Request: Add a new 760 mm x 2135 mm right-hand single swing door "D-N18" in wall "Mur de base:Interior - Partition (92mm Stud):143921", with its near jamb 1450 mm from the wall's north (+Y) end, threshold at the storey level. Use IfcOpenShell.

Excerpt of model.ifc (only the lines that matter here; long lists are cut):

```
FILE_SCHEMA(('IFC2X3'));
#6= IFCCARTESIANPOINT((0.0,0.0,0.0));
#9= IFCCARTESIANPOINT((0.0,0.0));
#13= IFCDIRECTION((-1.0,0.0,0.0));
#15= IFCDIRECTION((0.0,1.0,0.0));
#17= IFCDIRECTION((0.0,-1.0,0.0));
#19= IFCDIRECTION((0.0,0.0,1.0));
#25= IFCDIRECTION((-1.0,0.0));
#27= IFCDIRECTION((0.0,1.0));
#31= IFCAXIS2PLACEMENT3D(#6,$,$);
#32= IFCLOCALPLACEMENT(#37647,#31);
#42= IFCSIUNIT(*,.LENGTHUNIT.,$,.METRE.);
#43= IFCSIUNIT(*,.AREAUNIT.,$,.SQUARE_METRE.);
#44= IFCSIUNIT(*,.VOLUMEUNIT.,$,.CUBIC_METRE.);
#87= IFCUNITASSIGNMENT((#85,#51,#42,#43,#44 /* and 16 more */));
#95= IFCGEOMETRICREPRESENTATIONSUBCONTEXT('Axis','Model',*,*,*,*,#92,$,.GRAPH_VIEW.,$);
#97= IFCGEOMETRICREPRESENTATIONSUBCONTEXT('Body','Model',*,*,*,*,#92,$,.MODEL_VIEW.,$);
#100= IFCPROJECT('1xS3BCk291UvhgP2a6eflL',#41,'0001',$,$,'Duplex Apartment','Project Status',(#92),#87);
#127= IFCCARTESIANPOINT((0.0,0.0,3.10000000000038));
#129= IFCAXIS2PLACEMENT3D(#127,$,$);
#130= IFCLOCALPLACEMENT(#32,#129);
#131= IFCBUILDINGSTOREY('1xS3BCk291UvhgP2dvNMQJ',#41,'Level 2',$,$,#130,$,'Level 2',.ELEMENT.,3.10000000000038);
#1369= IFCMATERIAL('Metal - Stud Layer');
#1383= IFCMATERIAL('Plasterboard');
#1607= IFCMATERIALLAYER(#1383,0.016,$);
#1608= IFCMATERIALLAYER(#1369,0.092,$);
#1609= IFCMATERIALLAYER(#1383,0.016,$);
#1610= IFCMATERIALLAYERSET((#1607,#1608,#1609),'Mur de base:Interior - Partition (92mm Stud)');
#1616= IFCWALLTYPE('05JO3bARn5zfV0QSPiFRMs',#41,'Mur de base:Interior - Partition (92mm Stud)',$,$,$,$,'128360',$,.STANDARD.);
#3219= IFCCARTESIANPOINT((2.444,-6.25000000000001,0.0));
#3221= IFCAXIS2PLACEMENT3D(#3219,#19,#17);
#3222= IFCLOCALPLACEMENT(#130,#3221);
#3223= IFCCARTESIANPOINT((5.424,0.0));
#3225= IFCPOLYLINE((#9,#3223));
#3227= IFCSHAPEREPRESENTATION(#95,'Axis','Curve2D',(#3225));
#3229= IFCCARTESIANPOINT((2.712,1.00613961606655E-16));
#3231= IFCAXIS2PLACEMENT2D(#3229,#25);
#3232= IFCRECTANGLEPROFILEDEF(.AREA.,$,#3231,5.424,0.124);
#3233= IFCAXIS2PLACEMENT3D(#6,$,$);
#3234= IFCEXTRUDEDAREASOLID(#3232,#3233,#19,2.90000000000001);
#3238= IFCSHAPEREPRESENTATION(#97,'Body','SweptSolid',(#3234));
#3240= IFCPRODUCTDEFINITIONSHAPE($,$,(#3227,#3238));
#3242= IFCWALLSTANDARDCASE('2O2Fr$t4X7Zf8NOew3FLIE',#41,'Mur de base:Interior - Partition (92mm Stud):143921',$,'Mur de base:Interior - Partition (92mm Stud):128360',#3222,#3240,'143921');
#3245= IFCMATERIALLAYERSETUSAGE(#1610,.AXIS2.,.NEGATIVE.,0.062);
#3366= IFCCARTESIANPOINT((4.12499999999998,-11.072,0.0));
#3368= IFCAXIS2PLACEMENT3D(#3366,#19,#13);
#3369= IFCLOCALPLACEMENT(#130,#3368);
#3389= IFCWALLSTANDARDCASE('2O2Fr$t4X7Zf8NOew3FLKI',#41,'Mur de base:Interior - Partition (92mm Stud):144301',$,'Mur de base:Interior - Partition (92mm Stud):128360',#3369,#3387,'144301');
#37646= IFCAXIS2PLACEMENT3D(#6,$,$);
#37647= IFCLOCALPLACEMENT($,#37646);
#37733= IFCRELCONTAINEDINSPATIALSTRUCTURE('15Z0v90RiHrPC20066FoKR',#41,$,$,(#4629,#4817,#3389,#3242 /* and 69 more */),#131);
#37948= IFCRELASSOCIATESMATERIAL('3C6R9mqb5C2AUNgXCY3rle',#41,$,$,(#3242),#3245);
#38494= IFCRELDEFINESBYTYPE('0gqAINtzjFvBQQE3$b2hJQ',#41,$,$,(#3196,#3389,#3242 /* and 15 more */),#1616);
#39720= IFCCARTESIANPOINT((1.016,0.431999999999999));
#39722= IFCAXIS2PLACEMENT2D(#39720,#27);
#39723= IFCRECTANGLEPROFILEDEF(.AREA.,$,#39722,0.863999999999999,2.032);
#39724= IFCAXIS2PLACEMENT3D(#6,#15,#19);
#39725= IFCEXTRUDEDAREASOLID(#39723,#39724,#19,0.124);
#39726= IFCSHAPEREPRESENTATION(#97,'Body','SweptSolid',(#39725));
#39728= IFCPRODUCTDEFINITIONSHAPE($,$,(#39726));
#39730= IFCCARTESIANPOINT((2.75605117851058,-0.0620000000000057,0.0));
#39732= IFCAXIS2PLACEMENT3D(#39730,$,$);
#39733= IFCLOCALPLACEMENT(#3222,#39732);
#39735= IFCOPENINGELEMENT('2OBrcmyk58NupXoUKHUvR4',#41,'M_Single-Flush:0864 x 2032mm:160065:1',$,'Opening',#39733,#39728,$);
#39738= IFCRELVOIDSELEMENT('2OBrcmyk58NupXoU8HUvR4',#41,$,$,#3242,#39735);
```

```python
import numpy as np
import ifcopenshell
import ifcopenshell.api.feature
import ifcopenshell.api.geometry
import ifcopenshell.api.root
import ifcopenshell.api.spatial
import ifcopenshell.api.type
import ifcopenshell.geom
import ifcopenshell.util.element
import ifcopenshell.util.placement
import ifcopenshell.util.representation
import ifcopenshell.util.shape
import ifcopenshell.util.unit

model = ifcopenshell.open("model.ifc")
unit_scale = ifcopenshell.util.unit.calculate_unit_scale(model)
settings = ifcopenshell.geom.settings()


def volume(element):
    """Net volume in cubic metres, openings subtracted."""
    shape = ifcopenshell.geom.create_shape(settings, element)
    return ifcopenshell.util.shape.get_volume(shape.geometry)


wall = model.by_id(3242)
storey = ifcopenshell.util.element.get_container(wall, ifc_class="IfcBuildingStorey")
context = ifcopenshell.util.representation.get_context(model, "Model", "Body", "MODEL_VIEW")
before = volume(wall)

width, height, from_end, sill = 0.76, 2.135, 1.45, 0.0  # metres

# The wall runs along its own X axis, and the end named is its -X end.
wall_shape = ifcopenshell.geom.create_shape(settings, wall)
x, y, z = ifcopenshell.util.shape.get_vertices(wall_shape.geometry).T
start = x.min() + from_end
face, thickness = float(y.min()), float(y.max() - y.min())
wall_matrix = ifcopenshell.util.placement.get_local_placement(wall.ObjectPlacement)
level = ifcopenshell.util.placement.get_local_placement(storey.ObjectPlacement)[2, 3]


def in_wall(x, y):
    """Placement at x, y metres in the wall's axes, at sill height."""
    matrix = wall_matrix.copy()
    matrix[:, 3] = wall_matrix @ np.array([x / unit_scale, y / unit_scale, 0.0, 1.0])
    matrix[2, 3] = level + sill / unit_scale
    return matrix


# Opening: a box that overshoots both wall faces by 50 mm.
opening = ifcopenshell.api.root.create_entity(model, ifc_class="IfcOpeningElement")
box = ifcopenshell.api.geometry.add_wall_representation(
    model, context=context, length=width, height=height, thickness=thickness + 0.1
)
ifcopenshell.api.geometry.assign_representation(model, product=opening, representation=box)
ifcopenshell.api.geometry.edit_object_placement(model, product=opening, matrix=in_wall(start, face - 0.05), is_si=False)
ifcopenshell.api.feature.add_feature(model, feature=opening, element=wall)

door = ifcopenshell.api.root.create_entity(model, ifc_class="IfcDoor", name="D-N18")
door.OverallWidth, door.OverallHeight = width / unit_scale, height / unit_scale
body = ifcopenshell.api.geometry.add_door_representation(
    model,
    context=context,
    overall_width=door.OverallWidth,
    overall_height=door.OverallHeight,
    operation_type="SINGLE_SWING_RIGHT",
    lining_properties={"LiningDepth": thickness / unit_scale, "ThresholdDepth": thickness / unit_scale},
)
ifcopenshell.api.geometry.assign_representation(model, product=door, representation=body)
ifcopenshell.api.spatial.assign_container(model, products=[door], relating_structure=storey)
fills = ifcopenshell.api.feature.add_filling(model, opening=opening, element=door)
fills.OwnerHistory = door.OwnerHistory  # required in IFC2X3

# IFC2X3 keeps the operation on the door style.
style = ifcopenshell.api.root.create_entity(model, ifc_class="IfcDoorStyle", name="D-N18")
style.OperationType, style.ConstructionType = "SINGLE_SWING_RIGHT", "NOTDEFINED"
style.ParameterTakesPrecedence = style.Sizeable = False
ifcopenshell.api.type.assign_type(model, related_objects=[door], relating_type=style)

# The lining spans the wall, so the door starts at the wall face.
ifcopenshell.api.geometry.edit_object_placement(model, product=door, matrix=in_wall(start, face), is_si=False)

after = volume(wall)

print(f"wall volume {before:.3f} -> {after:.3f} m3")

model.write("model_edited.ifc")
```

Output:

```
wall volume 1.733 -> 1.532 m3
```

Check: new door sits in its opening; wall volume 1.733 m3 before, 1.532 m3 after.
